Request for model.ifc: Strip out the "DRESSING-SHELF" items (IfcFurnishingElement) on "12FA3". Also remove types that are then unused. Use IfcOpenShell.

First a look at what the model holds.

```python
import ifcopenshell
import ifcopenshell.util.element

model = ifcopenshell.open("model.ifc")
print(model.schema)
storey = next(s for s in model.by_type("IfcBuildingStorey") if s.Name == "12FA3")
furniture = [e for e in ifcopenshell.util.element.get_decomposition(storey) if e.is_a("IfcFurnishingElement")]
seen = {}
for e in furniture:
    element_type = ifcopenshell.util.element.get_type(e)
    name = element_type.Name if element_type not in (None, e) else None
    seen[name] = seen.get(name, 0) + 1
for name, count in sorted(seen.items(), key=str):
    print(count, "x", name)
```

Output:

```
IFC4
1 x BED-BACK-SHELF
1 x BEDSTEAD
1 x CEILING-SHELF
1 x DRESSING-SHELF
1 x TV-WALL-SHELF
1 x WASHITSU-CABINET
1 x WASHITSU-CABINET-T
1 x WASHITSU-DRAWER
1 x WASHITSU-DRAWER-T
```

```python
import ifcopenshell
import ifcopenshell.api.root
import ifcopenshell.util.element

model = ifcopenshell.open("model.ifc")

storey = next(s for s in model.by_type("IfcBuildingStorey") if s.Name == "12FA3")
furniture = [e for e in ifcopenshell.util.element.get_decomposition(storey) if e.is_a("IfcFurnishingElement")]
targets = [e for e in furniture if (t := ifcopenshell.util.element.get_type(e)) not in (None, e) and t.Name == "DRESSING-SHELF"]
types = {ifcopenshell.util.element.get_type(e) for e in targets} - {None, *targets}

for e in targets:
    ifcopenshell.api.root.remove_product(model, product=e)
print(len(targets), "removed")

unused = [t for t in types if not ifcopenshell.util.element.get_types(t)]
for t in unused:
    ifcopenshell.api.root.remove_product(model, product=t)
print(len(unused), "unused types removed")

model.write("model_v2.ifc")
```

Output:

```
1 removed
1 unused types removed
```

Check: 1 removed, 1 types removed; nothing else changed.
